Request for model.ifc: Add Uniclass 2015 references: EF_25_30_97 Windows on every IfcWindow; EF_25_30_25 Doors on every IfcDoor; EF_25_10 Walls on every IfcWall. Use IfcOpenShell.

First a look at what the model holds.

```python
import ifcopenshell

model = ifcopenshell.open("model.ifc")
print(model.schema)
print("classifications:", [c.Name for c in model.by_type("IfcClassification")])
for ifc_class in ("IfcDoor", "IfcRoof", "IfcStair", "IfcWall", "IfcWindow"):
    print(ifc_class, len(model.by_type(ifc_class)))
```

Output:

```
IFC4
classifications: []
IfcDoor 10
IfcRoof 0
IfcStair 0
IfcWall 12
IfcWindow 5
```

```python
import ifcopenshell
import ifcopenshell.api.classification

model = ifcopenshell.open("model.ifc")

system = ifcopenshell.api.classification.add_classification(model, classification="Uniclass 2015")

codes = {
    "IfcWindow": ("EF_25_30_97", "Windows"),
    "IfcDoor": ("EF_25_30_25", "Doors"),
    "IfcWall": ("EF_25_10", "Walls"),
}
for ifc_class, (code, name) in codes.items():
    products = model.by_type(ifc_class)
    ifcopenshell.api.classification.add_reference(
        model, products=products, classification=system, identification=code, name=name
    )
    print(code, len(products))

model.write("model_v2.ifc")
```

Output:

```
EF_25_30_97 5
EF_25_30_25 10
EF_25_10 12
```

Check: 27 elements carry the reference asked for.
